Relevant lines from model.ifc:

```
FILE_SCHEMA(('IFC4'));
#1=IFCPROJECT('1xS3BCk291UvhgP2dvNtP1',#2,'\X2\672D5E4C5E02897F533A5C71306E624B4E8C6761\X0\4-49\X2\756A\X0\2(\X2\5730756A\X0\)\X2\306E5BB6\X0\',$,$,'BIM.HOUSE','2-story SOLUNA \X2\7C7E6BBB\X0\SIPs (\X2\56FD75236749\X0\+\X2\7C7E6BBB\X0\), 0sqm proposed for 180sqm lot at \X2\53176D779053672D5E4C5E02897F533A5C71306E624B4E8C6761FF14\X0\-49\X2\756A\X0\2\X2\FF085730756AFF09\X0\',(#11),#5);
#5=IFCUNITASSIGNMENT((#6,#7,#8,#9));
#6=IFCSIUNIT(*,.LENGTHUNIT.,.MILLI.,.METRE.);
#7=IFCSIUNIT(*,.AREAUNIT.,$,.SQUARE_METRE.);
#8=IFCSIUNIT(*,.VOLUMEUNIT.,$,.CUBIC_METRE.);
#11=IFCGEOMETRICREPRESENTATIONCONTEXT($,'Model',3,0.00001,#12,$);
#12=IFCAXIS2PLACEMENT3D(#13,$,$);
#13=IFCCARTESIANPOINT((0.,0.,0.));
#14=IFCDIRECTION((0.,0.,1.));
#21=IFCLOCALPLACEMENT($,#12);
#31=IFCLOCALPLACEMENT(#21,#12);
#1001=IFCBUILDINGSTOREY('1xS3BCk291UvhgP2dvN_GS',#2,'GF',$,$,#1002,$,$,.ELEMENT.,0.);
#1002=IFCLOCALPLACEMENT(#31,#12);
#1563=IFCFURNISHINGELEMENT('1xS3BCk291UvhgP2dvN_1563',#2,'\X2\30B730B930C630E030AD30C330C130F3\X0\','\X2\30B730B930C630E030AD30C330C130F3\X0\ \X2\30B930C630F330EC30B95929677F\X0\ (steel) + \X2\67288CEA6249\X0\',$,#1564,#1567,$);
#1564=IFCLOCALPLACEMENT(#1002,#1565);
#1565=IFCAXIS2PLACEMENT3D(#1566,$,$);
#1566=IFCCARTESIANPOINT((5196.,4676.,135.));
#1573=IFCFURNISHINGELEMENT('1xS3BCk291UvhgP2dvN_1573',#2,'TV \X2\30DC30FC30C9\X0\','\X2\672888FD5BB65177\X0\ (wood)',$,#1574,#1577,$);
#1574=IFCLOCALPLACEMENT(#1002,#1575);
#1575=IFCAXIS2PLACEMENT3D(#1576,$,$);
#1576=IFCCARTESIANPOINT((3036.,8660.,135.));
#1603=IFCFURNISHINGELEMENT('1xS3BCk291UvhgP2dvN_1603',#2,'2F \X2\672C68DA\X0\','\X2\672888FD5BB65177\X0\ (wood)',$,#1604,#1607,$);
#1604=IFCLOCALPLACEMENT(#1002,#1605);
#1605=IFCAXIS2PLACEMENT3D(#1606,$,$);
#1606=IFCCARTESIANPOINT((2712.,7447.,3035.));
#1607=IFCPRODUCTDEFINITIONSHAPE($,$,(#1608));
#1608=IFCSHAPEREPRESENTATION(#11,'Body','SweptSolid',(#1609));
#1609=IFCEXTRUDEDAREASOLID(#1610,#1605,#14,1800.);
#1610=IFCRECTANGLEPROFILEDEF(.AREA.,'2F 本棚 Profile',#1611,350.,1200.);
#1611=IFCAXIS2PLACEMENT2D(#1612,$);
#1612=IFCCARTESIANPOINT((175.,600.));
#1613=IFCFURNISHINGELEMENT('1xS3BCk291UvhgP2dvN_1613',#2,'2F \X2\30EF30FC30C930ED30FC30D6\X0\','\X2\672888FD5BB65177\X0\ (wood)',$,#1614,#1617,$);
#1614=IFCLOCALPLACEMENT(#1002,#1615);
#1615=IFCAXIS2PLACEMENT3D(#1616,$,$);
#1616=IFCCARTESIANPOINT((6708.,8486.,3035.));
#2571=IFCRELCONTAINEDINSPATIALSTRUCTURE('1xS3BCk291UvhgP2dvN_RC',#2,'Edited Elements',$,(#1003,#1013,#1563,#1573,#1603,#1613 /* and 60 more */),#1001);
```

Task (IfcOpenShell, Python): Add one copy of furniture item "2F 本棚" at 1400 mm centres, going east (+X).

```python
import numpy as np
import ifcopenshell
import ifcopenshell.api.geometry
import ifcopenshell.api.root
import ifcopenshell.util.element
import ifcopenshell.util.placement

model = ifcopenshell.open("model.ifc")


def reuse_history(source, copy):
    """copy_class also copies each property set's owner history, people and application; keep the originals."""
    for rel in copy.IsDefinedBy:
        if rel.is_a("IfcRelDefinesByProperties") and (history := rel.RelatingPropertyDefinition.OwnerHistory):
            rel.RelatingPropertyDefinition.OwnerHistory = source.OwnerHistory
            ifcopenshell.util.element.remove_deep2(model, history)


source = model.by_guid("1xS3BCk291UvhgP2dvN_1603")
base = ifcopenshell.util.placement.get_local_placement(source.ObjectPlacement)
step = np.array([1.0, 0.0, 0.0]) * 1400.0

for i in range(1, 2):
    copy = ifcopenshell.api.root.copy_class(model, product=source)
    copy.Representation = ifcopenshell.util.element.copy_deep(
        model, source.Representation, exclude=["IfcGeometricRepresentationContext", "IfcRepresentationMap"]
    )
    reuse_history(source, copy)
    matrix = base.copy()
    matrix[:3, 3] += i * step
    print("added at", matrix[:3, 3].round(3) + 0.0)
    ifcopenshell.api.geometry.edit_object_placement(model, product=copy, matrix=matrix, is_si=False)

model.write("model_rev.ifc")
```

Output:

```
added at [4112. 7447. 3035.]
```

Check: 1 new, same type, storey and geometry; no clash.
